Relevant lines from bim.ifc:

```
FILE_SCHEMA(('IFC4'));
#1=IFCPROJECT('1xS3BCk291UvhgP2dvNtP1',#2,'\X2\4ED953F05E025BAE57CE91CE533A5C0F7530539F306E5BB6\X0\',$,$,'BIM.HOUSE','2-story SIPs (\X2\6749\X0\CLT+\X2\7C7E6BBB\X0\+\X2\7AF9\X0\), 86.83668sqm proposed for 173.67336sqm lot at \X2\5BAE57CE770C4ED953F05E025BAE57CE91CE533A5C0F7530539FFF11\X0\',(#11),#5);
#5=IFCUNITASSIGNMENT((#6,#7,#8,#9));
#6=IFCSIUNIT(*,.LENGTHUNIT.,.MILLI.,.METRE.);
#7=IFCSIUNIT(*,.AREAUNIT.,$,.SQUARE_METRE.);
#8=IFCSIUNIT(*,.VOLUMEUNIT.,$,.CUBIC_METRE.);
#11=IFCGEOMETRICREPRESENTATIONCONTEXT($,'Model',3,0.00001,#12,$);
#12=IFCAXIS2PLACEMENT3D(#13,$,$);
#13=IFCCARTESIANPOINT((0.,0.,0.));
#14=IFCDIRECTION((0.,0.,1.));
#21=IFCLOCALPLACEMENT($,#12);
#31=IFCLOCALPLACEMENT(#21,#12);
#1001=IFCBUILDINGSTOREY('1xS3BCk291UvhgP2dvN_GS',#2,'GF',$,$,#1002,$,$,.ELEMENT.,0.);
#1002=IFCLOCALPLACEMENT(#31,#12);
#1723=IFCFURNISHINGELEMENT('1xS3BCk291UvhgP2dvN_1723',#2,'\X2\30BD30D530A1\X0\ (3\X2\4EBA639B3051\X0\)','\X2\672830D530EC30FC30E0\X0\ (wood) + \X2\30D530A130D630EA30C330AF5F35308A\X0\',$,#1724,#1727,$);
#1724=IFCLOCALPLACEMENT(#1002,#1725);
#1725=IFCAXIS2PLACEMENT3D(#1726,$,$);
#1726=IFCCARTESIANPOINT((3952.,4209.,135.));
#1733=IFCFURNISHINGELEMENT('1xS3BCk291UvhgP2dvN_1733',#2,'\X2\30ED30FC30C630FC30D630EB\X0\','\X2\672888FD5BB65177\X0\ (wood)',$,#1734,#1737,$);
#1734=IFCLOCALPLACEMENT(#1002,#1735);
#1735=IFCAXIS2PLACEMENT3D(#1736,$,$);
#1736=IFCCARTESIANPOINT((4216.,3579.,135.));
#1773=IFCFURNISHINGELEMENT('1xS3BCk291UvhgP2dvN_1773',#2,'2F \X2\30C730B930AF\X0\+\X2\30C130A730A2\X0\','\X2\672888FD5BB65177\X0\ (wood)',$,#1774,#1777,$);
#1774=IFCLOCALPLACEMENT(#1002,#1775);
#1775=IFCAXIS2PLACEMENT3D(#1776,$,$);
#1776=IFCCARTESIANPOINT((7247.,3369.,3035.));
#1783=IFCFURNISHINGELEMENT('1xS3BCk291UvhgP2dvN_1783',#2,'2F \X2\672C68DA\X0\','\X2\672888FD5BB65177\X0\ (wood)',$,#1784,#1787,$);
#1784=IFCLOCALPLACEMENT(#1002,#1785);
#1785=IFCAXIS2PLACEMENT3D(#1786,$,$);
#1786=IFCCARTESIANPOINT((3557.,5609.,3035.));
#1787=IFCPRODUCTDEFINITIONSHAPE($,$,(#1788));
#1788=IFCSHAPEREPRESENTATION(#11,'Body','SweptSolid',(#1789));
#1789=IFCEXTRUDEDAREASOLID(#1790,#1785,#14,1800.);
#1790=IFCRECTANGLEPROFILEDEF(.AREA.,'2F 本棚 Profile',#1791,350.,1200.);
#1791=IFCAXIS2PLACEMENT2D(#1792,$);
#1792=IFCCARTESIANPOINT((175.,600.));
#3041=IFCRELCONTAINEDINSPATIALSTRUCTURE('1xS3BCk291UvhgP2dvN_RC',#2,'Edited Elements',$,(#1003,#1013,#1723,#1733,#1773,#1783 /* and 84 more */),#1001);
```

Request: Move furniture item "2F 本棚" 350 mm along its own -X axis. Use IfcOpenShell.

```python
import ifcopenshell
import ifcopenshell.api.geometry
import ifcopenshell.util.placement
import ifcopenshell.util.unit

model = ifcopenshell.open("bim.ifc")
unit_scale = ifcopenshell.util.unit.calculate_unit_scale(model)

item = model.by_id(1783)
matrix = ifcopenshell.util.placement.get_local_placement(item.ObjectPlacement)
matrix[:3, 3] -= matrix[:3, 0] * 0.35 / unit_scale
ifcopenshell.api.geometry.edit_object_placement(model, product=item, matrix=matrix, is_si=False)

print(ifcopenshell.util.placement.get_local_placement(item.ObjectPlacement).round(3) + 0.0)

model.write("bim_v2.ifc")
```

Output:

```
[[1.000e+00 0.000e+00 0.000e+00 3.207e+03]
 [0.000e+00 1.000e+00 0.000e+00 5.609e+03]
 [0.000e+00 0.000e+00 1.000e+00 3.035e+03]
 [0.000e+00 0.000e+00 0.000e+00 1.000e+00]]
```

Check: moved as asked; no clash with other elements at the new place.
